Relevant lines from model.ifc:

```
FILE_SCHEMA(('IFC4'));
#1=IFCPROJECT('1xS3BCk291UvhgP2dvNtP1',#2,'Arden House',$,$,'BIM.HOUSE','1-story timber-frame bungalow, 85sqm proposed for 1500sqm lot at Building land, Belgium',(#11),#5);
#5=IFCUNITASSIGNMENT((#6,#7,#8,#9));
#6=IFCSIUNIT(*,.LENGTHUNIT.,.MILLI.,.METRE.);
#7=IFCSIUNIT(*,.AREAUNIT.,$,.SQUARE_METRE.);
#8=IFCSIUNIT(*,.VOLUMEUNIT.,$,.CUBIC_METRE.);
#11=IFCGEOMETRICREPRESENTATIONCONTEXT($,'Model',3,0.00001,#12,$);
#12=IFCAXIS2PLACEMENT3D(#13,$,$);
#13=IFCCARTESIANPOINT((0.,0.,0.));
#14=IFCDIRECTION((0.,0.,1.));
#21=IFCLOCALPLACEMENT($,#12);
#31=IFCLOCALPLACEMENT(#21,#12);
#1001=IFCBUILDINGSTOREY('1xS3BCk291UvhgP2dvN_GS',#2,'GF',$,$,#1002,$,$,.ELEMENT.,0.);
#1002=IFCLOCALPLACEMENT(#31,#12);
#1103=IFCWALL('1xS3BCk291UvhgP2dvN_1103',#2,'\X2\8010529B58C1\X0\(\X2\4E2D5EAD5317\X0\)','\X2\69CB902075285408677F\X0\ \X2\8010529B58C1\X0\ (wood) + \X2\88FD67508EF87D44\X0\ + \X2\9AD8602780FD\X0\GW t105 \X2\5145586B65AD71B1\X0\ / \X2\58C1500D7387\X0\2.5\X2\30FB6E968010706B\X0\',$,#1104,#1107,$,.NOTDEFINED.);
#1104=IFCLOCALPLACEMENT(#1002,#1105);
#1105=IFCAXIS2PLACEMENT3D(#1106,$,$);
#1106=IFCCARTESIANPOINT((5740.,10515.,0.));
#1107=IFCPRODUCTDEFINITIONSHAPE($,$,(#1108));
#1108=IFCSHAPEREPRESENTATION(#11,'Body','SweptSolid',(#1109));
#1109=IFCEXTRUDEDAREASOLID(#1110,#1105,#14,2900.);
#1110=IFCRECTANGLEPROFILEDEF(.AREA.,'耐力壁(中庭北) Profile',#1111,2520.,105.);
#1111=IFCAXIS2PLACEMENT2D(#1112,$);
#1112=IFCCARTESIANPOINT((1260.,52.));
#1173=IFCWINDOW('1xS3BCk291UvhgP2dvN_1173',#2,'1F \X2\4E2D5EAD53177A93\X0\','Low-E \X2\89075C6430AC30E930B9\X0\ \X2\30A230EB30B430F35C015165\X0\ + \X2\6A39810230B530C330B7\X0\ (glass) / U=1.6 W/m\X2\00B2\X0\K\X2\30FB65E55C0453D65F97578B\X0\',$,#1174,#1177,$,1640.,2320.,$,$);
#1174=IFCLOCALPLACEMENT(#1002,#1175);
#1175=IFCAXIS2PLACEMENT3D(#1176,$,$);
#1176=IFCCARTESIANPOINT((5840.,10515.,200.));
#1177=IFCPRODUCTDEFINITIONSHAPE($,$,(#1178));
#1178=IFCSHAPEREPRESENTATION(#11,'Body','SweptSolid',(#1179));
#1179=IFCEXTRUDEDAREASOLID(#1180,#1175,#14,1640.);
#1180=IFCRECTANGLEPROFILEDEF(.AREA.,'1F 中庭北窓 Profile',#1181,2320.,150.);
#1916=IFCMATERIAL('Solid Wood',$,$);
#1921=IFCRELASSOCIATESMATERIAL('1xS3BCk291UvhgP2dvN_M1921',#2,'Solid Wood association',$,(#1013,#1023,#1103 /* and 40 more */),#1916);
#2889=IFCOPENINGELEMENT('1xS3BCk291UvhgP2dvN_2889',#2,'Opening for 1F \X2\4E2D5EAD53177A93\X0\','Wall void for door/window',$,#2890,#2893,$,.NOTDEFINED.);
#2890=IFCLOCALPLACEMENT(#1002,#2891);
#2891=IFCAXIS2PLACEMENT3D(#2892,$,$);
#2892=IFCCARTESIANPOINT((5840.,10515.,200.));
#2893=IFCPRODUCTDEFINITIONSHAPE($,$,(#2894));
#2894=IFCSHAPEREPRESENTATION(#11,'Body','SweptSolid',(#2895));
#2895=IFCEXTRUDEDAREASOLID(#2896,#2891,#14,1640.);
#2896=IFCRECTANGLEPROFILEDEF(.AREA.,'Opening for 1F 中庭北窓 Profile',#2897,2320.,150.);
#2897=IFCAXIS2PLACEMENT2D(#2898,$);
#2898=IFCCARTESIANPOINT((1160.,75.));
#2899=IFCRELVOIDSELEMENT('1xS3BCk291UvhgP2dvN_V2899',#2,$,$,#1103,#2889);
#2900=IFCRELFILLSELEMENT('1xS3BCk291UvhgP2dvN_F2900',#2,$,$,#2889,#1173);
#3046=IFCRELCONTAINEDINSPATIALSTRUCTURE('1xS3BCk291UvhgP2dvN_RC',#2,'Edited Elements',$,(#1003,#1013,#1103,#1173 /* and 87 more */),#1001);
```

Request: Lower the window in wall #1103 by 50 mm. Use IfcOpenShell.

```python
import numpy as np
import ifcopenshell
import ifcopenshell.api.geometry
import ifcopenshell.util.placement
import ifcopenshell.util.unit

model = ifcopenshell.open("model.ifc")
unit_scale = ifcopenshell.util.unit.calculate_unit_scale(model)

window = model.by_guid("1xS3BCk291UvhgP2dvN_1173")
opening = window.FillsVoids[0].RelatingOpeningElement
dz = -0.05 / unit_scale

shift = np.array([0.0, 0.0, dz])
# The window is not placed relative to its opening, so move both.
for product in (opening, window):
    matrix = ifcopenshell.util.placement.get_local_placement(product.ObjectPlacement)
    matrix[:3, 3] += shift
    ifcopenshell.api.geometry.edit_object_placement(model, product=product, matrix=matrix, is_si=False)

print(f"moved by {dz * unit_scale:+.3f} m")

model.write("model_edited.ifc")
```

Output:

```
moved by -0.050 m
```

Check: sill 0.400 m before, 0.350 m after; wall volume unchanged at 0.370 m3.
